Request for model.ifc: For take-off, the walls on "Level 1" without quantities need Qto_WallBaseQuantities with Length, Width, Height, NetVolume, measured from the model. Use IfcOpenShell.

First a look at what the model holds.

```python
import ifcopenshell
import ifcopenshell.util.element
import ifcopenshell.util.unit

model = ifcopenshell.open("model.ifc")
print(model.schema)
for unit_type in ("LENGTHUNIT", "AREAUNIT", "VOLUMEUNIT"):
    print(unit_type, ifcopenshell.util.unit.calculate_unit_scale(model, unit_type))
storey = next(s for s in model.by_type("IfcBuildingStorey") if s.Name == "Level 1")
walls = [e for e in ifcopenshell.util.element.get_decomposition(storey) if e.is_a("IfcWall")]
for e in sorted(walls, key=lambda e: e.id()):
    print(e.id(), e.is_a(), e.Name, list(ifcopenshell.util.element.get_psets(e, qtos_only=True)), sep=" | ")
```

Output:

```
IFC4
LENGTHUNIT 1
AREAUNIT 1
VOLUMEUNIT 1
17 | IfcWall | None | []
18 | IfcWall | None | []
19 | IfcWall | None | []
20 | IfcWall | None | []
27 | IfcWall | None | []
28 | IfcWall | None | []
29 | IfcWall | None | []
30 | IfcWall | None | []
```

```python
import ifcopenshell
import ifcopenshell.api.pset
import ifcopenshell.geom
import ifcopenshell.util.element
import ifcopenshell.util.shape
import ifcopenshell.util.unit

model = ifcopenshell.open("model.ifc")
unit_scale = ifcopenshell.util.unit.calculate_unit_scale(model)
volume_scale = ifcopenshell.util.unit.calculate_unit_scale(model, "VOLUMEUNIT")
settings = ifcopenshell.geom.settings()

storey = next(s for s in model.by_type("IfcBuildingStorey") if s.Name == "Level 1")
walls = [e for e in ifcopenshell.util.element.get_decomposition(storey) if e.is_a("IfcWall")]

for e in sorted(walls, key=lambda e: e.id()):
    if ifcopenshell.util.element.get_psets(e, qtos_only=True, should_inherit=False):
        continue
    # Geometry comes back in metres, in the element's own axes.
    shape = ifcopenshell.geom.create_shape(settings, e)
    values = {
        "Length": ifcopenshell.util.shape.get_x(shape.geometry) / unit_scale,
        "Width": ifcopenshell.util.shape.get_y(shape.geometry) / unit_scale,
        "Height": ifcopenshell.util.shape.get_z(shape.geometry) / unit_scale,
        "NetVolume": ifcopenshell.util.shape.get_volume(shape.geometry) / volume_scale,
    }
    qto = ifcopenshell.api.pset.add_qto(model, product=e, name="Qto_WallBaseQuantities")
    ifcopenshell.api.pset.edit_qto(model, qto=qto, properties=values)
    print(e.id(), {k: round(v, 3) for k, v in values.items()})

model.write("model_updated.ifc")
```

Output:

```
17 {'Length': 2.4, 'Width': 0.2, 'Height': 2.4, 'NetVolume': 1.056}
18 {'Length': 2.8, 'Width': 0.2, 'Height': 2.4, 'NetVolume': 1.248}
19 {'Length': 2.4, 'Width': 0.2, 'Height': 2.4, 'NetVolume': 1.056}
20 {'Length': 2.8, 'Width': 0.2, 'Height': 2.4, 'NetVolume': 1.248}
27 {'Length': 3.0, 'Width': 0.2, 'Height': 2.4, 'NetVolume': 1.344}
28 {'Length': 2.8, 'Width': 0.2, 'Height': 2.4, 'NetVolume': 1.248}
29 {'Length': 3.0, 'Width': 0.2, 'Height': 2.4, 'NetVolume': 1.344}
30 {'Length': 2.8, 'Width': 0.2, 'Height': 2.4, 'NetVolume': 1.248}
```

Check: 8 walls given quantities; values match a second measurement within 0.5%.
